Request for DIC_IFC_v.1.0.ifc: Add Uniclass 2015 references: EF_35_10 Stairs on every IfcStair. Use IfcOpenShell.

First a look at what the model holds.

```python
import ifcopenshell

model = ifcopenshell.open("DIC_IFC_v.1.0.ifc")
print(model.schema)
print("classifications:", [c.Name for c in model.by_type("IfcClassification")])
for ifc_class in ("IfcDoor", "IfcRoof", "IfcStair", "IfcWall", "IfcWindow"):
    print(ifc_class, len(model.by_type(ifc_class)))
```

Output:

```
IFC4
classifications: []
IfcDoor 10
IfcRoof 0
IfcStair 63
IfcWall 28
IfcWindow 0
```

```python
import ifcopenshell
import ifcopenshell.api.classification

model = ifcopenshell.open("DIC_IFC_v.1.0.ifc")

system = ifcopenshell.api.classification.add_classification(model, classification="Uniclass 2015")

codes = {
    "IfcStair": ("EF_35_10", "Stairs"),
}
for ifc_class, (code, name) in codes.items():
    products = model.by_type(ifc_class)
    ifcopenshell.api.classification.add_reference(
        model, products=products, classification=system, identification=code, name=name
    )
    print(code, len(products))

model.write("DIC_IFC_v.1.0_edited.ifc")
```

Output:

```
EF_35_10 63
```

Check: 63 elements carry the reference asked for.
